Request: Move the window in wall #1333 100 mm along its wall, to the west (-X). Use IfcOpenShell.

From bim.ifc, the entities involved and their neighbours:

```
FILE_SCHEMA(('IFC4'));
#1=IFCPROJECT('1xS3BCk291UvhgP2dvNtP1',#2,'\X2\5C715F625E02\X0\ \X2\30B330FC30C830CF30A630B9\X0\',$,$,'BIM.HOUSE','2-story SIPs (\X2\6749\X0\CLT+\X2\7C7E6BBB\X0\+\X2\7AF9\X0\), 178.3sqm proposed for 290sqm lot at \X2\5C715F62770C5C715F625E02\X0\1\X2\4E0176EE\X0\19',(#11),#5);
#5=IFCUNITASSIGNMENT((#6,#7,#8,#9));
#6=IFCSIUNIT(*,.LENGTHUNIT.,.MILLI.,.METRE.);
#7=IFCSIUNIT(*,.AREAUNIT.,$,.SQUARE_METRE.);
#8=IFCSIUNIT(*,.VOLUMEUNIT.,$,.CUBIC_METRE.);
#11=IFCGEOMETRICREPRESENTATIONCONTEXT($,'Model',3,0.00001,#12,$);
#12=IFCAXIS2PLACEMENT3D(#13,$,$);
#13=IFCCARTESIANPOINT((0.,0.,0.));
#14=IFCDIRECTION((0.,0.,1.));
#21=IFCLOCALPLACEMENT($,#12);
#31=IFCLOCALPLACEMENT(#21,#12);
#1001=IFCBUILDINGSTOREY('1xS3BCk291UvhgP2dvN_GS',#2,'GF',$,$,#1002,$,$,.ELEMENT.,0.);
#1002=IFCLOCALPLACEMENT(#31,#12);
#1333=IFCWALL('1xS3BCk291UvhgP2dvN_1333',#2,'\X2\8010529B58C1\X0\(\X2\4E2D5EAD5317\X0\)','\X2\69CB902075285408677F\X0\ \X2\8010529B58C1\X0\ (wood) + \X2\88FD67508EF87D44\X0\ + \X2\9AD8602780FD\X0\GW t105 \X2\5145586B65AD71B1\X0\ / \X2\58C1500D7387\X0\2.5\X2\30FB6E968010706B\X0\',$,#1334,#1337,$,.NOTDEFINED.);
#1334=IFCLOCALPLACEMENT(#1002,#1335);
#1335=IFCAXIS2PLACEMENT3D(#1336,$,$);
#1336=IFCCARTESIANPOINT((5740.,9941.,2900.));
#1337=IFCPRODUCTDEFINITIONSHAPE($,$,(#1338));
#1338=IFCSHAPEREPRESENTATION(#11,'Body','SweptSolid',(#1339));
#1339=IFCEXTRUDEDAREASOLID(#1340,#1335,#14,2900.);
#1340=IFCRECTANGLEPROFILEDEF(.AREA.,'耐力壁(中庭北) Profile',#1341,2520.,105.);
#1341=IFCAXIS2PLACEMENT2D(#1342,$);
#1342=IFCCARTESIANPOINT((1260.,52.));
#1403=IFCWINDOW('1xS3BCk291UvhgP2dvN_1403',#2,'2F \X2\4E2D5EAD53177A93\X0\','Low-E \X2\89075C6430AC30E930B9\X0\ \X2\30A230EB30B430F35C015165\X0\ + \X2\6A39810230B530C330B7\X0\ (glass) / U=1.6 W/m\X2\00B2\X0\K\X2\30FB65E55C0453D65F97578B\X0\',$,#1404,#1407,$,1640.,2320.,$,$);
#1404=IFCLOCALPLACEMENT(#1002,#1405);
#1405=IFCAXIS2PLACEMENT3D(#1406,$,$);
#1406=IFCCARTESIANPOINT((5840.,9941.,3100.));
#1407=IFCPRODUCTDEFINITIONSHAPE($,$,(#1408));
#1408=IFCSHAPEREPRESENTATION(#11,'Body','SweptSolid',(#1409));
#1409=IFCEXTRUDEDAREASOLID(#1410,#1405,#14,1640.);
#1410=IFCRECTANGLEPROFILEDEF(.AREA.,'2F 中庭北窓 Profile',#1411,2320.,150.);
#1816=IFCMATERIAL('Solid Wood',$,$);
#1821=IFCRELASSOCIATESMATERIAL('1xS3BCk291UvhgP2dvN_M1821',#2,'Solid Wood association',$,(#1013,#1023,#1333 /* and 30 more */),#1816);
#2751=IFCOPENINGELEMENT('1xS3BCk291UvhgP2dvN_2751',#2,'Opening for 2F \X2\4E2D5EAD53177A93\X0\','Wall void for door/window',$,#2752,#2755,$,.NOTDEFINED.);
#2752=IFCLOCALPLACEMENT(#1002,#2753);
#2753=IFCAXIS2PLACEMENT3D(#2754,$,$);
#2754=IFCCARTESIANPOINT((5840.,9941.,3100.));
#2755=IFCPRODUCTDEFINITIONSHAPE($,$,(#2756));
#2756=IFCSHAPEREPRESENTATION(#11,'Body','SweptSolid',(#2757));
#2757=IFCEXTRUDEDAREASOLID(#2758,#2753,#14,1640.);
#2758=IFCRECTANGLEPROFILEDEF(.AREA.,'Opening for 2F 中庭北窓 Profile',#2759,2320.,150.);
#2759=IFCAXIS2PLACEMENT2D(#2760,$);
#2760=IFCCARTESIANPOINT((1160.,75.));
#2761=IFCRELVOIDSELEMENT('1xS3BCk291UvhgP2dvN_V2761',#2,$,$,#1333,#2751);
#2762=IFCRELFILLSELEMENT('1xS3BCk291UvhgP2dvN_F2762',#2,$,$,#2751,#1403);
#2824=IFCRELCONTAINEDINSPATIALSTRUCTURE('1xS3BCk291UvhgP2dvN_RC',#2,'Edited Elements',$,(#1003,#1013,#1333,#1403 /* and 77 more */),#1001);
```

```python
import ifcopenshell
import ifcopenshell.api.geometry
import ifcopenshell.util.placement
import ifcopenshell.util.unit

model = ifcopenshell.open("bim.ifc")
unit_scale = ifcopenshell.util.unit.calculate_unit_scale(model)

window = model.by_guid("1xS3BCk291UvhgP2dvN_1403")
opening = window.FillsVoids[0].RelatingOpeningElement
wall = opening.VoidsElements[0].RelatingBuildingElement

wall_matrix = ifcopenshell.util.placement.get_local_placement(wall.ObjectPlacement)
shift = wall_matrix[:3, 0] * -0.1 / unit_scale
before = ifcopenshell.util.placement.get_local_placement(window.ObjectPlacement)[:3, 3].copy()

# The window is not placed relative to its opening, so move both.
for product in (opening, window):
    matrix = ifcopenshell.util.placement.get_local_placement(product.ObjectPlacement)
    matrix[:3, 3] += shift
    ifcopenshell.api.geometry.edit_object_placement(model, product=product, matrix=matrix, is_si=False)

after = ifcopenshell.util.placement.get_local_placement(window.ObjectPlacement)[:3, 3]
print("window moved by", (after - before).round(3) + 0.0)

model.write("bim_updated.ifc")
```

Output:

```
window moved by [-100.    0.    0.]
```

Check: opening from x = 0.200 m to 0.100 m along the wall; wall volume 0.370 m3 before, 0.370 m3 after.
